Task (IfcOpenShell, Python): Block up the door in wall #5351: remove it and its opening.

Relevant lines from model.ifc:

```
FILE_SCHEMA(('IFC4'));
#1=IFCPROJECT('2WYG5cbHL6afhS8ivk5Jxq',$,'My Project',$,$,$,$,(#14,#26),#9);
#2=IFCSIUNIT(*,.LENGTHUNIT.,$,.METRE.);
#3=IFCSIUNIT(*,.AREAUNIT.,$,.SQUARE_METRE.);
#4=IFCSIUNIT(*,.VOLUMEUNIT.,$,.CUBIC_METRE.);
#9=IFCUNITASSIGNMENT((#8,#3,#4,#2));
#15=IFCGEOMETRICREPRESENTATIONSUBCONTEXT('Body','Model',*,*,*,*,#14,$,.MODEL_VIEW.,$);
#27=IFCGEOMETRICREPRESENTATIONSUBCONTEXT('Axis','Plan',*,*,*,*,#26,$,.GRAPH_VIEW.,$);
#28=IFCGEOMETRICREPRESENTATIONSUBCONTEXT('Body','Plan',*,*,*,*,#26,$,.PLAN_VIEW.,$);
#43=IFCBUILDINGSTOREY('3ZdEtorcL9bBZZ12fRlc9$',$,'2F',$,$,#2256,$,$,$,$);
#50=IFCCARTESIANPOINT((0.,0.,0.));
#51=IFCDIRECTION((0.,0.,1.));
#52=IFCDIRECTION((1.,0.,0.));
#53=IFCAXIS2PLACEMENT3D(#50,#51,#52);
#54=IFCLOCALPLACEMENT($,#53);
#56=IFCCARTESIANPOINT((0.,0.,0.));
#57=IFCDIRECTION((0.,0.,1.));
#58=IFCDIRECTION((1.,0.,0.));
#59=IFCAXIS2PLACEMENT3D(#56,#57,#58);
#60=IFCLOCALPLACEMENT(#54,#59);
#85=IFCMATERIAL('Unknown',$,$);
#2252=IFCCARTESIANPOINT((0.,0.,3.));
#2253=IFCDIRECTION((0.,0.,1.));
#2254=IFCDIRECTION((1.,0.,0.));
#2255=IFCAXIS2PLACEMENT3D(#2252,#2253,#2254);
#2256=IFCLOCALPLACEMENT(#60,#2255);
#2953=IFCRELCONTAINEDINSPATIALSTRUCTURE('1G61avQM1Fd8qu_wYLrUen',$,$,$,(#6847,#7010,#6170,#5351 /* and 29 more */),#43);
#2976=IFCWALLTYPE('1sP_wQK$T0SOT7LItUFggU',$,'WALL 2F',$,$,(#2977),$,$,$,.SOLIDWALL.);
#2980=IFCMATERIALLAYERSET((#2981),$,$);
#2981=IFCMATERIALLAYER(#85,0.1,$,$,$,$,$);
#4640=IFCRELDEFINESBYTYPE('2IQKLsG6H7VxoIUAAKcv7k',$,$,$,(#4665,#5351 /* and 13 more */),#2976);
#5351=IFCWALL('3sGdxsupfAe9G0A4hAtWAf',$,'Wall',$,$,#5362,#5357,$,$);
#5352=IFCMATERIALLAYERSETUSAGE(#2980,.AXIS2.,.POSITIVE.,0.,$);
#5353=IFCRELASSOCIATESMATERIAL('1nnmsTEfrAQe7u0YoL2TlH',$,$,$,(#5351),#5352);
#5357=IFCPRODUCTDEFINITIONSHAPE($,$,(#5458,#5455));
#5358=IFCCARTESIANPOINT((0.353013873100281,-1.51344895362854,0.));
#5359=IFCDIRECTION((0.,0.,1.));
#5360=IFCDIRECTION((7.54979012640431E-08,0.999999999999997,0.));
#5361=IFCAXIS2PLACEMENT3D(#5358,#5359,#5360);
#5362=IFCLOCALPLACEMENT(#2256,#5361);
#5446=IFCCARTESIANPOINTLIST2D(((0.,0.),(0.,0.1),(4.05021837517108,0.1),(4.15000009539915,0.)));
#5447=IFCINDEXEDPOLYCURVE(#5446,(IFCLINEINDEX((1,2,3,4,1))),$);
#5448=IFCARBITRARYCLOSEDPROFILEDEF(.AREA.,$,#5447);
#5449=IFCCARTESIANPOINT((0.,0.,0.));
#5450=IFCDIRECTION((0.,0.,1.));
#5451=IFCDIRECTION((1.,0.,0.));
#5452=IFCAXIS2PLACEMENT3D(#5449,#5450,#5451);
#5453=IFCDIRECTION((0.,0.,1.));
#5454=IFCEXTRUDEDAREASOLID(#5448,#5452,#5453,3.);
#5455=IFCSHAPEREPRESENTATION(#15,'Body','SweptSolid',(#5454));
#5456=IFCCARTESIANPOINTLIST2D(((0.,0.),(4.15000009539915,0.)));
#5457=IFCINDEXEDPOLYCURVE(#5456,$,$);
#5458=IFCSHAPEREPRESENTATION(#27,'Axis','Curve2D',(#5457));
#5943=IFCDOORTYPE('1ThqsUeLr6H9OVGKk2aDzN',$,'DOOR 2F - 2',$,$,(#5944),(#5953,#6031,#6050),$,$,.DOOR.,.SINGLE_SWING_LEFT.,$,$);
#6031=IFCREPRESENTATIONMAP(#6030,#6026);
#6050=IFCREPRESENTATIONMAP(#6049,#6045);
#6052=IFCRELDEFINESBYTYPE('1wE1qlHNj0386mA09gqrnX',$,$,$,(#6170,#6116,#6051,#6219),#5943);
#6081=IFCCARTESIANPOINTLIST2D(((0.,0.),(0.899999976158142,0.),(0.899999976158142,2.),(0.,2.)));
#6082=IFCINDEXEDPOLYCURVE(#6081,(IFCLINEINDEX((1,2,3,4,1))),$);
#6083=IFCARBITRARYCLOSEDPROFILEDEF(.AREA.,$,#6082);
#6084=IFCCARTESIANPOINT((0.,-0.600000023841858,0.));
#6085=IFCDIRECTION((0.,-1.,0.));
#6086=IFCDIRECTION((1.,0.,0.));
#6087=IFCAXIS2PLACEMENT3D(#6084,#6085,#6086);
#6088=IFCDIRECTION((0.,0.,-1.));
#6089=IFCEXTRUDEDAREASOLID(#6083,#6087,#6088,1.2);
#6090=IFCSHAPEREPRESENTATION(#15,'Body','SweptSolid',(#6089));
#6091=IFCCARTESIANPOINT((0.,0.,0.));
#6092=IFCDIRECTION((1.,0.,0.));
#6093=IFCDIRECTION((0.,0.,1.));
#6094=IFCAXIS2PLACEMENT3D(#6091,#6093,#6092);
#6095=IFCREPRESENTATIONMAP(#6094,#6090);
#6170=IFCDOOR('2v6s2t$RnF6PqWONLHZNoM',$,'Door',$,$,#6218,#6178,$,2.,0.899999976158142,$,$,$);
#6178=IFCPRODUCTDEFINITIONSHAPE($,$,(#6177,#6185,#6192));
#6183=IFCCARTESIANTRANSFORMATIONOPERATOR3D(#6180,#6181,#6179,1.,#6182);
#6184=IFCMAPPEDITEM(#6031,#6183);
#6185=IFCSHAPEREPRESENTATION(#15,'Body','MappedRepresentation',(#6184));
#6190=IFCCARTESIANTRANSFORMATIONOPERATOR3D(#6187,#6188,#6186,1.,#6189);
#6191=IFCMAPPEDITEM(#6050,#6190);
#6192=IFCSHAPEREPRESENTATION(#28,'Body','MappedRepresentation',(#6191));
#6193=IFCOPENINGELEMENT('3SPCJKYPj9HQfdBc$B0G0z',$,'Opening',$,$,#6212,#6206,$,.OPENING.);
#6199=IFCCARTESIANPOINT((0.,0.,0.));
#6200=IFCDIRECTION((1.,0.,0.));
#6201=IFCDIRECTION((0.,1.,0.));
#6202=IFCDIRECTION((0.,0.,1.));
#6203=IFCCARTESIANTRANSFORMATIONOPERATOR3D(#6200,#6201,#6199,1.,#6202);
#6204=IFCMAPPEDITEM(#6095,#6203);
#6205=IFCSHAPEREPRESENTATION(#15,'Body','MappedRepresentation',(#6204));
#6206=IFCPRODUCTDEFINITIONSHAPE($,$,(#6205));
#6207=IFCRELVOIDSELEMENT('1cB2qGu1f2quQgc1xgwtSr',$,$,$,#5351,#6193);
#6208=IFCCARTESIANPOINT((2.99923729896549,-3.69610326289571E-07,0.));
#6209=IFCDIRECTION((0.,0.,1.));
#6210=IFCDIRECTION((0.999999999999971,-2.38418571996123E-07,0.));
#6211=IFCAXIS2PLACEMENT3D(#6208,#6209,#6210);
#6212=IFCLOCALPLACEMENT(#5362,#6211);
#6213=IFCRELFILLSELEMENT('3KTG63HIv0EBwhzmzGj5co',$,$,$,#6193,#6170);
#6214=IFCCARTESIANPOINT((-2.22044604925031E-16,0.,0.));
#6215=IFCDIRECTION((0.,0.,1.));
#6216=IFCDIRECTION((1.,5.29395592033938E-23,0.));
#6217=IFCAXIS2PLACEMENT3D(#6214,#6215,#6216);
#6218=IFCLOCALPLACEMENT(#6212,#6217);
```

```python
import ifcopenshell
import ifcopenshell.api.feature
import ifcopenshell.api.root
import ifcopenshell.geom
import ifcopenshell.util.shape

model = ifcopenshell.open("model.ifc")
settings = ifcopenshell.geom.settings()


def volume(element):
    """Net volume in cubic metres, openings subtracted."""
    shape = ifcopenshell.geom.create_shape(settings, element)
    return ifcopenshell.util.shape.get_volume(shape.geometry)


door = model.by_guid("2v6s2t$RnF6PqWONLHZNoM")
opening = door.FillsVoids[0].RelatingOpeningElement
wall = opening.VoidsElements[0].RelatingBuildingElement
before = volume(wall)

ifcopenshell.api.root.remove_product(model, product=door)
ifcopenshell.api.feature.remove_feature(model, feature=opening)

after = volume(wall)

print(f"wall volume {before:.3f} -> {after:.3f} m3")

model.write("model_edited.ifc")
```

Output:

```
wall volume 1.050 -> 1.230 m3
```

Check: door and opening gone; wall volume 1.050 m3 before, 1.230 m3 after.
